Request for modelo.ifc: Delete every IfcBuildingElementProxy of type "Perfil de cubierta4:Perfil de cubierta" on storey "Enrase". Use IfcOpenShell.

First a look at what the model holds.

```python
import ifcopenshell
import ifcopenshell.util.element

model = ifcopenshell.open("modelo.ifc")
print(model.schema)
storey = next(s for s in model.by_type("IfcBuildingStorey") if s.Name == "Enrase")
proxies = [e for e in ifcopenshell.util.element.get_decomposition(storey) if e.is_a("IfcBuildingElementProxy")]
seen = {}
for e in proxies:
    element_type = ifcopenshell.util.element.get_type(e)
    name = element_type.Name if element_type not in (None, e) else None
    seen[name] = seen.get(name, 0) + 1
for name, count in sorted(seen.items(), key=str):
    print(count, "x", name)
```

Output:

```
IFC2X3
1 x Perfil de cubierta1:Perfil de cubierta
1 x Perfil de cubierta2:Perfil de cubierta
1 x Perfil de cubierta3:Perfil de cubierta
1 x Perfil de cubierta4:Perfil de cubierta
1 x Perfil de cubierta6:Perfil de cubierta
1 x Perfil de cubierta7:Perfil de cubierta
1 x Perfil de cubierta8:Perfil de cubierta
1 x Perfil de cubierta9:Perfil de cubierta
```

```python
import ifcopenshell
import ifcopenshell.api.root
import ifcopenshell.util.element

model = ifcopenshell.open("modelo.ifc")

storey = next(s for s in model.by_type("IfcBuildingStorey") if s.Name == "Enrase")
proxies = [e for e in ifcopenshell.util.element.get_decomposition(storey) if e.is_a("IfcBuildingElementProxy")]
targets = [e for e in proxies if (t := ifcopenshell.util.element.get_type(e)) not in (None, e) and t.Name == "Perfil de cubierta4:Perfil de cubierta"]

for e in targets:
    ifcopenshell.api.root.remove_product(model, product=e)
print(len(targets), "removed")

model.write("modelo_v2.ifc")
```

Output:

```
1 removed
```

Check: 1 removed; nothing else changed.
